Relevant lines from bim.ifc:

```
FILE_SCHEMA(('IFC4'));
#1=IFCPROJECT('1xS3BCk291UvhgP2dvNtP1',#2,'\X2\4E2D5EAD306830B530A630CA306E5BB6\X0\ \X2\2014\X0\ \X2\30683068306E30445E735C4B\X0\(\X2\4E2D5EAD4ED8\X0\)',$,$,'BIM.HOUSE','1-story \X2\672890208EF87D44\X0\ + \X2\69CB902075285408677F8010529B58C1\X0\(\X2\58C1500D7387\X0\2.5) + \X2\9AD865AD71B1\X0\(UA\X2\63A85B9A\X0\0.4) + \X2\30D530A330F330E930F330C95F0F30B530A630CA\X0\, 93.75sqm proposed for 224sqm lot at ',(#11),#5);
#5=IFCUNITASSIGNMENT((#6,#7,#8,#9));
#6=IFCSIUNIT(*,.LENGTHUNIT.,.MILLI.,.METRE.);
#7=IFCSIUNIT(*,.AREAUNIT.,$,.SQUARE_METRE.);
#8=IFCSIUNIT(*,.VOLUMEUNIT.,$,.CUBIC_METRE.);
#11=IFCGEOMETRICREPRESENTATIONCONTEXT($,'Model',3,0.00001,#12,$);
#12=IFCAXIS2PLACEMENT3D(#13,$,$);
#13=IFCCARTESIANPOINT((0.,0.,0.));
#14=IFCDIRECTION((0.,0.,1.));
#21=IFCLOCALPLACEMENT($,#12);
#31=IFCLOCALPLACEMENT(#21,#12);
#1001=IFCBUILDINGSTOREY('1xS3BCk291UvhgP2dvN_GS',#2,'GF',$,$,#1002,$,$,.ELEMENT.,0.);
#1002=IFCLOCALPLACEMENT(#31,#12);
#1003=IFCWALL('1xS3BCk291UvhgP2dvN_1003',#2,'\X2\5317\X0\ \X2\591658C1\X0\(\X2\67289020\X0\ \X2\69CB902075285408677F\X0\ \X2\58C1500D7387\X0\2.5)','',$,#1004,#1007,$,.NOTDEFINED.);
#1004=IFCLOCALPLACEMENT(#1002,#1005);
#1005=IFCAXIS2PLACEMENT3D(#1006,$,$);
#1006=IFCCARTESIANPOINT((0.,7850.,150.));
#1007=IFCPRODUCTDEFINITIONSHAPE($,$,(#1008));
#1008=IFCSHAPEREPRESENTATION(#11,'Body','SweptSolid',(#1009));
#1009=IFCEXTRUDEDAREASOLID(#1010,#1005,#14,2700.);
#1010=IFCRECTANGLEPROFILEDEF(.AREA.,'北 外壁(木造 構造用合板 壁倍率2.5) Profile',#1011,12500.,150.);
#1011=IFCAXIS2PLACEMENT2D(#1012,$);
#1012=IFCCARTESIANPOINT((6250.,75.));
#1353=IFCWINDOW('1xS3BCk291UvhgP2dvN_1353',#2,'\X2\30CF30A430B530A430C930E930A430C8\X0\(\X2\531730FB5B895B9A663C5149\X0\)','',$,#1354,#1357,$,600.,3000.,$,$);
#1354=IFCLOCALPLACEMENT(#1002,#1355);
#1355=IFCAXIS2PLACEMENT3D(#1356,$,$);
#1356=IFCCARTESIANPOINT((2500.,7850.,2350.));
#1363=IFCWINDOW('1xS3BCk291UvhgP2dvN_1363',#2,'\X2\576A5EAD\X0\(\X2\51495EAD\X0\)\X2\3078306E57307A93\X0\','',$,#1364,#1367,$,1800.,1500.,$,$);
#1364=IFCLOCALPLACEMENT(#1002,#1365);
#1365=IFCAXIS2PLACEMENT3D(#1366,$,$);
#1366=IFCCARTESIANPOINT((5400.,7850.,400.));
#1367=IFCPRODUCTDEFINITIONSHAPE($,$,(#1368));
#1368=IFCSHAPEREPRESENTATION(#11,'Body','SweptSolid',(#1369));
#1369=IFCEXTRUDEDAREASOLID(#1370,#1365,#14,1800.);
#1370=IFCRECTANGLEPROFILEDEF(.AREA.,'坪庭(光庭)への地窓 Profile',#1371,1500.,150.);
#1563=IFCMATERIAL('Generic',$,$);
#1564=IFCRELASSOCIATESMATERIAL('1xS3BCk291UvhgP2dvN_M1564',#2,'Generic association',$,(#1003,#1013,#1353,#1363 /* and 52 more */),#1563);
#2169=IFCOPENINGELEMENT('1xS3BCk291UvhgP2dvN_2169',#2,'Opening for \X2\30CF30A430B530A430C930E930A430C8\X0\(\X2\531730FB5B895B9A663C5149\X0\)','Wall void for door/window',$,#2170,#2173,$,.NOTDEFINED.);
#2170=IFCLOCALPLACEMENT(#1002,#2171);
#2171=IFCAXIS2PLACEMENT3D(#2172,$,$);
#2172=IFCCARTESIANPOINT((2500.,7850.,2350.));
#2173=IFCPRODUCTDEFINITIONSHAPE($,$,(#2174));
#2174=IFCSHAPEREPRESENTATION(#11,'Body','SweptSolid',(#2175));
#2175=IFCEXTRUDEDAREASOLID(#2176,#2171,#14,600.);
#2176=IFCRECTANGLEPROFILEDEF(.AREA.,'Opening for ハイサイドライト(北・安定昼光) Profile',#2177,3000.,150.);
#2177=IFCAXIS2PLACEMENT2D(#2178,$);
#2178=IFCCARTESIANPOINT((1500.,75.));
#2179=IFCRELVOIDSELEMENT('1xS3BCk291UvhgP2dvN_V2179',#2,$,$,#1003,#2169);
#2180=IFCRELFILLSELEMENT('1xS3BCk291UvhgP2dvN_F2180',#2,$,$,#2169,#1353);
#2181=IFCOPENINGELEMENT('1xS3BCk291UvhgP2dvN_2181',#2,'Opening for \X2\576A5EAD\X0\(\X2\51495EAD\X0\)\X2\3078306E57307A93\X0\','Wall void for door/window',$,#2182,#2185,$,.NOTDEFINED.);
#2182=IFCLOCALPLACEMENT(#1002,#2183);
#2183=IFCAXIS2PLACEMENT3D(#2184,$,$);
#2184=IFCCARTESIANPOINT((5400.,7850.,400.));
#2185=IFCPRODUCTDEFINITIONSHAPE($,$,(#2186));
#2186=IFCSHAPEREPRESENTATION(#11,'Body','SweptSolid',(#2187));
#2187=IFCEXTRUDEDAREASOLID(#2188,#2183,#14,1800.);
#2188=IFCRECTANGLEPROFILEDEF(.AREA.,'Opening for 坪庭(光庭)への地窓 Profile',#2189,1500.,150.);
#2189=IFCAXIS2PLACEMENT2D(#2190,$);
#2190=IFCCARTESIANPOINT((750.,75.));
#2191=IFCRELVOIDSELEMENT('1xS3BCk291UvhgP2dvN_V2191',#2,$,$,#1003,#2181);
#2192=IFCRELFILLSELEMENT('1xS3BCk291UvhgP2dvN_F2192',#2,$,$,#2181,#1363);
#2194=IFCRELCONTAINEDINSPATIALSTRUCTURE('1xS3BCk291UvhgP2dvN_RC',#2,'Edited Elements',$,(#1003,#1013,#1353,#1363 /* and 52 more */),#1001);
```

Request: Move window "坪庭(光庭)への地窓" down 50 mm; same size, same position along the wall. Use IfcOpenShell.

```python
import numpy as np
import ifcopenshell
import ifcopenshell.api.geometry
import ifcopenshell.util.placement
import ifcopenshell.util.unit

model = ifcopenshell.open("bim.ifc")
unit_scale = ifcopenshell.util.unit.calculate_unit_scale(model)

window = model.by_id(1363)
opening = window.FillsVoids[0].RelatingOpeningElement
dz = -0.05 / unit_scale

shift = np.array([0.0, 0.0, dz])
# The window is not placed relative to its opening, so move both.
for product in (opening, window):
    matrix = ifcopenshell.util.placement.get_local_placement(product.ObjectPlacement)
    matrix[:3, 3] += shift
    ifcopenshell.api.geometry.edit_object_placement(model, product=product, matrix=matrix, is_si=False)

print(f"moved by {dz * unit_scale:+.3f} m")

model.write("bim_edited.ifc")
```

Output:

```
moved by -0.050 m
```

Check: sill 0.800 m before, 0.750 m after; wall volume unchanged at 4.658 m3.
